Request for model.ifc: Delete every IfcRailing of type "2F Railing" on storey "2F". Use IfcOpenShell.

First a look at what the model holds.

```python
import ifcopenshell
import ifcopenshell.util.element

model = ifcopenshell.open("model.ifc")
print(model.schema)
storey = next(s for s in model.by_type("IfcBuildingStorey") if s.Name == "2F")
railings = [e for e in ifcopenshell.util.element.get_decomposition(storey) if e.is_a("IfcRailing")]
seen = {}
for e in railings:
    element_type = ifcopenshell.util.element.get_type(e)
    name = element_type.Name if element_type not in (None, e) else None
    seen[name] = seen.get(name, 0) + 1
for name, count in sorted(seen.items(), key=str):
    print(count, "x", name)
```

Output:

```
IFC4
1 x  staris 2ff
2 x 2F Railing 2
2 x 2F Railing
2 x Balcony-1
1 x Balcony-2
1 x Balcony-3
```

```python
import ifcopenshell
import ifcopenshell.api.root
import ifcopenshell.util.element

model = ifcopenshell.open("model.ifc")

storey = next(s for s in model.by_type("IfcBuildingStorey") if s.Name == "2F")
railings = [e for e in ifcopenshell.util.element.get_decomposition(storey) if e.is_a("IfcRailing")]
targets = [e for e in railings if (t := ifcopenshell.util.element.get_type(e)) not in (None, e) and t.Name == "2F Railing"]

for e in targets:
    ifcopenshell.api.root.remove_product(model, product=e)
print(len(targets), "removed")

model.write("model_v2.ifc")
```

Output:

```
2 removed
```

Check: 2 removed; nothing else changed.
